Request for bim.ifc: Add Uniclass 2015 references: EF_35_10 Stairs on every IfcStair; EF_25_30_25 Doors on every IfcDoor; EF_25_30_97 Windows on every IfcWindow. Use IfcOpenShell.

First a look at what the model holds.

```python
import ifcopenshell

model = ifcopenshell.open("bim.ifc")
print(model.schema)
print("classifications:", [c.Name for c in model.by_type("IfcClassification")])
for ifc_class in ("IfcDoor", "IfcRoof", "IfcStair", "IfcWall", "IfcWindow"):
    print(ifc_class, len(model.by_type(ifc_class)))
```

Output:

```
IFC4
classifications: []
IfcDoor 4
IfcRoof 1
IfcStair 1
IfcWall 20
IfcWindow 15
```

```python
import ifcopenshell
import ifcopenshell.api.classification

model = ifcopenshell.open("bim.ifc")

system = ifcopenshell.api.classification.add_classification(model, classification="Uniclass 2015")

codes = {
    "IfcStair": ("EF_35_10", "Stairs"),
    "IfcDoor": ("EF_25_30_25", "Doors"),
    "IfcWindow": ("EF_25_30_97", "Windows"),
}
for ifc_class, (code, name) in codes.items():
    products = model.by_type(ifc_class)
    ifcopenshell.api.classification.add_reference(
        model, products=products, classification=system, identification=code, name=name
    )
    print(code, len(products))

model.write("bim_edited.ifc")
```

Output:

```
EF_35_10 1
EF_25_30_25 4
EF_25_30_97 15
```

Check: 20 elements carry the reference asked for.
